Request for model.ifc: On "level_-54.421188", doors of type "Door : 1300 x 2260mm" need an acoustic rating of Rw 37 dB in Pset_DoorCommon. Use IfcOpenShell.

First a look at what the model holds.

```python
import ifcopenshell
import ifcopenshell.util.element

model = ifcopenshell.open("model.ifc")
print(model.schema)
storey = next(s for s in model.by_type("IfcBuildingStorey") if s.Name == "level_-54.421188")
doors = [e for e in ifcopenshell.util.element.get_decomposition(storey) if e.is_a("IfcDoor")]
seen = {}
for e in doors:
    element_type = ifcopenshell.util.element.get_type(e)
    key = (element_type.Name if element_type != e and element_type else None, ifcopenshell.util.element.get_pset(e, "Pset_DoorCommon", "AcousticRating"))
    seen[key] = seen.get(key, 0) + 1
for (name, value), count in sorted(seen.items(), key=str):
    print(count, "x", name, "|", value)
```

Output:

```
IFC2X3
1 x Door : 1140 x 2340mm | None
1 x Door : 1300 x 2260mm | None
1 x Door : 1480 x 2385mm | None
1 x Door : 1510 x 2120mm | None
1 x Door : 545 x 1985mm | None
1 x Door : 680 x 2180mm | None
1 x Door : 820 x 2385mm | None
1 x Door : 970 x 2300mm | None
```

```python
import ifcopenshell
import ifcopenshell.api.pset
import ifcopenshell.util.element

model = ifcopenshell.open("model.ifc")

storey = next(s for s in model.by_type("IfcBuildingStorey") if s.Name == "level_-54.421188")
doors = [e for e in ifcopenshell.util.element.get_decomposition(storey) if e.is_a("IfcDoor")]

count = 0
for e in doors:
    element_type = ifcopenshell.util.element.get_type(e)
    if element_type in (None, e) or element_type.Name != "Door : 1300 x 2260mm":
        continue
    # add_pset returns the element's existing set when there is one.
    pset = ifcopenshell.api.pset.add_pset(model, product=e, name="Pset_DoorCommon")
    ifcopenshell.api.pset.edit_pset(model, pset=pset, properties={"AcousticRating": "Rw 37 dB"})
    count += 1

print(count, "doors updated")

model.write("model_v2.ifc")
```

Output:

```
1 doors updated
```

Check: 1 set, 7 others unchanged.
